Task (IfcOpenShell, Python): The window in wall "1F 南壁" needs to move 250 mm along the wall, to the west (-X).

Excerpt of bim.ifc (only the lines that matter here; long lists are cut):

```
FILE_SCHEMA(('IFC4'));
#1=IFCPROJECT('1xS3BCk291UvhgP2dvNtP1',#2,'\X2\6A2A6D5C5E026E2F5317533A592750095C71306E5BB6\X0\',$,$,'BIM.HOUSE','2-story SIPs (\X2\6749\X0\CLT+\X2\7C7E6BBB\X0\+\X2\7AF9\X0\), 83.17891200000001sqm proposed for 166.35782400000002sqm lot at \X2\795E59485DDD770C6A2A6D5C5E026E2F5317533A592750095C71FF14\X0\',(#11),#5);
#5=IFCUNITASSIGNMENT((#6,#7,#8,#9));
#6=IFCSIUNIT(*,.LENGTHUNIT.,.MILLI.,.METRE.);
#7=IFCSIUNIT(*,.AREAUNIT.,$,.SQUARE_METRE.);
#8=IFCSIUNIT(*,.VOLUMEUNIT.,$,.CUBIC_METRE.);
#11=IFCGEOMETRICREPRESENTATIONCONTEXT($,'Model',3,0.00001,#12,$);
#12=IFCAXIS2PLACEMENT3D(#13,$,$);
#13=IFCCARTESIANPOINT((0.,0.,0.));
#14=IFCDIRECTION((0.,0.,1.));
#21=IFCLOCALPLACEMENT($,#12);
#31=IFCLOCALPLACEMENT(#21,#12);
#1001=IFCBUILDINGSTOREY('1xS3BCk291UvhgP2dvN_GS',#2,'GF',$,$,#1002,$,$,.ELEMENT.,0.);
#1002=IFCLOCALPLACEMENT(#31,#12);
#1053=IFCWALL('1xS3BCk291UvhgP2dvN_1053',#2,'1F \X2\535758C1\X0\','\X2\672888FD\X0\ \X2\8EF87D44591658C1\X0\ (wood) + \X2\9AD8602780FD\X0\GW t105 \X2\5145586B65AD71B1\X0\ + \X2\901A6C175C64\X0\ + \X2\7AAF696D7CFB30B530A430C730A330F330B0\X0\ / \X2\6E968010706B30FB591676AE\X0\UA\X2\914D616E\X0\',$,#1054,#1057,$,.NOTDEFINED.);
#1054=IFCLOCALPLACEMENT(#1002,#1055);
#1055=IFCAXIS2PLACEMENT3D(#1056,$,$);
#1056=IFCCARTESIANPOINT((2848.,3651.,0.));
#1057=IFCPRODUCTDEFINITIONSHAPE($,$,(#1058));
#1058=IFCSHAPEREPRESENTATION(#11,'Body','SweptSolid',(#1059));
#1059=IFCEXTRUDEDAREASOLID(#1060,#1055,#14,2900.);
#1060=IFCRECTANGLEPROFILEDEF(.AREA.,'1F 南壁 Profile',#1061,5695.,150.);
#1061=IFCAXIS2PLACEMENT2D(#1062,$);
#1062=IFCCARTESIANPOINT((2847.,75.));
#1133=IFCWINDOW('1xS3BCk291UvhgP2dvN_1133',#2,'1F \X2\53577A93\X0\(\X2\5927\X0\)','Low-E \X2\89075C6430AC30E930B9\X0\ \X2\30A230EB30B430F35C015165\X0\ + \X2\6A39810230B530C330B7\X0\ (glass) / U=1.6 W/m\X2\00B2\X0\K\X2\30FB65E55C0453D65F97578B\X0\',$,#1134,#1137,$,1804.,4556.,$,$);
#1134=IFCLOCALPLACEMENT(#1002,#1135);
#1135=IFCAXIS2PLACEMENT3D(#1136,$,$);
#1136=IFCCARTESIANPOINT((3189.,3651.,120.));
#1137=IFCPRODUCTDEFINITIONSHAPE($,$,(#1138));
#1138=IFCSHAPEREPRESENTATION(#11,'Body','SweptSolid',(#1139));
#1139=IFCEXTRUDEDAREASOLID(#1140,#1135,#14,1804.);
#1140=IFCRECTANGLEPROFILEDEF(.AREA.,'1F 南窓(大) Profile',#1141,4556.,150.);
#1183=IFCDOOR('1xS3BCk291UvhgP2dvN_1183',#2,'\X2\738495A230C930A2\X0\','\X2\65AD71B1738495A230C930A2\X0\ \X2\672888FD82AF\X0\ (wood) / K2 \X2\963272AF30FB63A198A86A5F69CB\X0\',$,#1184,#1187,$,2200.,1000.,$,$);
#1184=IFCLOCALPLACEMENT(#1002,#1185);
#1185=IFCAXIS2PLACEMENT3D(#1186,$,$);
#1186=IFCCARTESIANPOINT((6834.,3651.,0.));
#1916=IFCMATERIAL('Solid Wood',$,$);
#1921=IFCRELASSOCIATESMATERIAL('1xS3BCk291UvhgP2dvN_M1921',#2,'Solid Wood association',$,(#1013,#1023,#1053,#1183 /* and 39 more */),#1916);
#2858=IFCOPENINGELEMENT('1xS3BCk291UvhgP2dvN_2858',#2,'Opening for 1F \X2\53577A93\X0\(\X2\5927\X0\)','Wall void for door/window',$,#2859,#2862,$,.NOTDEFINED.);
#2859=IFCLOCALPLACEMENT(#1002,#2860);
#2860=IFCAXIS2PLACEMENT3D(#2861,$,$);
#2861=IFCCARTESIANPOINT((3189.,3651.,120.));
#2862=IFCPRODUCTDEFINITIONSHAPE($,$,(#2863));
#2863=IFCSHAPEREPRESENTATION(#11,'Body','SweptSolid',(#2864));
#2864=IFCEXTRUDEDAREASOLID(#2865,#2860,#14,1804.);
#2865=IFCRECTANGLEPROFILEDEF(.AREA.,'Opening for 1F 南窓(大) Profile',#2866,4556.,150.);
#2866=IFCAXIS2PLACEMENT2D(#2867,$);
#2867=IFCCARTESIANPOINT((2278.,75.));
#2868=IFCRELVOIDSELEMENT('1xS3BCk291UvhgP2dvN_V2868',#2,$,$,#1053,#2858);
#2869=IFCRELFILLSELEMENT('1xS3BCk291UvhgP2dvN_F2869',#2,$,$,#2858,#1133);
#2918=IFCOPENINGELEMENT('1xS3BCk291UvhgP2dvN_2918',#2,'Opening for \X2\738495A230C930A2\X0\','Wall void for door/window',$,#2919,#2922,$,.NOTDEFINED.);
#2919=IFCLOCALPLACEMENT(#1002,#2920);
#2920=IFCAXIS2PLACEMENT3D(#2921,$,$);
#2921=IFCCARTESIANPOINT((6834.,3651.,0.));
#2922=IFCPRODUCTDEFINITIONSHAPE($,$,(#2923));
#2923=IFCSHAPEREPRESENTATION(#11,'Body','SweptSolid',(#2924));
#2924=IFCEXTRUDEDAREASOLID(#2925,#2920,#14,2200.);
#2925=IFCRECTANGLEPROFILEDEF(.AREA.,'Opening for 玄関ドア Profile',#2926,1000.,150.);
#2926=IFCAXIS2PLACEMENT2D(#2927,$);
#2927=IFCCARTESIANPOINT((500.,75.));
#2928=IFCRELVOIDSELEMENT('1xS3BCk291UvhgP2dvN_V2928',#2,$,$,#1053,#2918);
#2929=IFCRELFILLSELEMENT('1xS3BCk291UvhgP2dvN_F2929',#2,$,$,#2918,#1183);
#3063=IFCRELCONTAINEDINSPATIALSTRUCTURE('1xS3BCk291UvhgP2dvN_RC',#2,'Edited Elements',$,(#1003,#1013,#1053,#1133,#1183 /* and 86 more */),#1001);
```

```python
import ifcopenshell
import ifcopenshell.api.geometry
import ifcopenshell.util.placement
import ifcopenshell.util.unit

model = ifcopenshell.open("bim.ifc")
unit_scale = ifcopenshell.util.unit.calculate_unit_scale(model)

window = model.by_id(1133)
opening = window.FillsVoids[0].RelatingOpeningElement
wall = opening.VoidsElements[0].RelatingBuildingElement

wall_matrix = ifcopenshell.util.placement.get_local_placement(wall.ObjectPlacement)
shift = wall_matrix[:3, 0] * -0.25 / unit_scale
before = ifcopenshell.util.placement.get_local_placement(window.ObjectPlacement)[:3, 3].copy()

# The window is not placed relative to its opening, so move both.
for product in (opening, window):
    matrix = ifcopenshell.util.placement.get_local_placement(product.ObjectPlacement)
    matrix[:3, 3] += shift
    ifcopenshell.api.geometry.edit_object_placement(model, product=product, matrix=matrix, is_si=False)

after = ifcopenshell.util.placement.get_local_placement(window.ObjectPlacement)[:3, 3]
print("window moved by", (after - before).round(3) + 0.0)

model.write("bim_edited.ifc")
```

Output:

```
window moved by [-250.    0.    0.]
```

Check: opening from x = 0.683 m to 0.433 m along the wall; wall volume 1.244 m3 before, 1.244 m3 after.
